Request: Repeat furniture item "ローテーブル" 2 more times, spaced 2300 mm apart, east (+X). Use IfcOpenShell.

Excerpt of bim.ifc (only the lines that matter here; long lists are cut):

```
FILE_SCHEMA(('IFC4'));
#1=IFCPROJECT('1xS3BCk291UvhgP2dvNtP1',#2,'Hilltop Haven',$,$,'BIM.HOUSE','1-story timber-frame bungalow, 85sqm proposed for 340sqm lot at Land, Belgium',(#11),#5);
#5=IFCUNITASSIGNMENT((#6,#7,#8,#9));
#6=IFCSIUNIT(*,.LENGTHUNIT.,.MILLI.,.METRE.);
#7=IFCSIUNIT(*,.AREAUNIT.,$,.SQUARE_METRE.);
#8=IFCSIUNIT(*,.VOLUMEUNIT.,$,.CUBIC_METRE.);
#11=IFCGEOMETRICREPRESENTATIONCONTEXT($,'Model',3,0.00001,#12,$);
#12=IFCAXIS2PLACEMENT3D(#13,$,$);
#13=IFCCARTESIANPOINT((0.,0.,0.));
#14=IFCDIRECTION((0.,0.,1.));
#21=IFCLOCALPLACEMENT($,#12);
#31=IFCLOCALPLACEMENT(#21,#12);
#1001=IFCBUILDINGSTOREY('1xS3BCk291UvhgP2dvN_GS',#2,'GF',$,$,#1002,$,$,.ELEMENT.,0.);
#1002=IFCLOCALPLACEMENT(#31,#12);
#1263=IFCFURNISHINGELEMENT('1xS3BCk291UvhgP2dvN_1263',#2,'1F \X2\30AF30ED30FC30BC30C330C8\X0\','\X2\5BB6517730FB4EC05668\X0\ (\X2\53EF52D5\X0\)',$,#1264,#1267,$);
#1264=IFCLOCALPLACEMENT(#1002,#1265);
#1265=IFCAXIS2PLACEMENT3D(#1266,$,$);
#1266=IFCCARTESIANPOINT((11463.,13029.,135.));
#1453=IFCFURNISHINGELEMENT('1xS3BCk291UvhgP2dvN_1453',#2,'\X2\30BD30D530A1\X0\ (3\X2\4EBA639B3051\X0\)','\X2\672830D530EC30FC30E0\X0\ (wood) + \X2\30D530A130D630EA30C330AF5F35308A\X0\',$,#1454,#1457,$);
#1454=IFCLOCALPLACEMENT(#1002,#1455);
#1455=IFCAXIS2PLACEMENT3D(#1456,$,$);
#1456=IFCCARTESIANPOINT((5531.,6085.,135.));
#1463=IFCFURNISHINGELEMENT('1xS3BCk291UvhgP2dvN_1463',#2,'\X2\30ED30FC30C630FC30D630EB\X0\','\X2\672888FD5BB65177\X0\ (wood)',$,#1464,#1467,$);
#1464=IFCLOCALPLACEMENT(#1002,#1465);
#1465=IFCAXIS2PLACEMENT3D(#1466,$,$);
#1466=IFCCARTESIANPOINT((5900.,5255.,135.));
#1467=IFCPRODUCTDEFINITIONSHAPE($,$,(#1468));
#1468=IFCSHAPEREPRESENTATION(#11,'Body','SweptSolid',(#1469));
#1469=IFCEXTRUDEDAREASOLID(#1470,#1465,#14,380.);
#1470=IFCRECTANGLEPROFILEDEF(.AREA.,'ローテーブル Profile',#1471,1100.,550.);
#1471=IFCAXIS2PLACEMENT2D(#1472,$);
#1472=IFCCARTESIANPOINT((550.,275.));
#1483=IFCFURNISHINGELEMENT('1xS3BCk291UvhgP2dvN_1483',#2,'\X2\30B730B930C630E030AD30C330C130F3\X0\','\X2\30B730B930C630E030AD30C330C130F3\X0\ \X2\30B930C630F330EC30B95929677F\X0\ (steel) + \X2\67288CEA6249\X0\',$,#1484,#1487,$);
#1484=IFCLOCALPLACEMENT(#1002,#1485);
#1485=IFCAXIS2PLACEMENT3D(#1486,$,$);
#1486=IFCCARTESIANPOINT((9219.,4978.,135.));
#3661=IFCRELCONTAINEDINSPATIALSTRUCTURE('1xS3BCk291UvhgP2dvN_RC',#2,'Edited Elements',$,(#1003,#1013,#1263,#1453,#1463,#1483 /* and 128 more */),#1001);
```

```python
import numpy as np
import ifcopenshell
import ifcopenshell.api.geometry
import ifcopenshell.api.root
import ifcopenshell.util.element
import ifcopenshell.util.placement
import ifcopenshell.util.unit

model = ifcopenshell.open("bim.ifc")
unit_scale = ifcopenshell.util.unit.calculate_unit_scale(model)


def reuse_history(source, copy):
    """copy_class also copies each property set's owner history, people and application; keep the originals."""
    for rel in copy.IsDefinedBy:
        if rel.is_a("IfcRelDefinesByProperties") and (history := rel.RelatingPropertyDefinition.OwnerHistory):
            rel.RelatingPropertyDefinition.OwnerHistory = source.OwnerHistory
            ifcopenshell.util.element.remove_deep2(model, history)


source = model.by_guid("1xS3BCk291UvhgP2dvN_1463")
base = ifcopenshell.util.placement.get_local_placement(source.ObjectPlacement)
step = np.array([1.0, 0.0, 0.0]) * 2.3 / unit_scale

for i in range(1, 3):
    copy = ifcopenshell.api.root.copy_class(model, product=source)
    copy.Representation = ifcopenshell.util.element.copy_deep(
        model, source.Representation, exclude=["IfcGeometricRepresentationContext", "IfcRepresentationMap"]
    )
    reuse_history(source, copy)
    matrix = base.copy()
    matrix[:3, 3] += i * step
    print("added at", matrix[:3, 3].round(3) + 0.0)
    ifcopenshell.api.geometry.edit_object_placement(model, product=copy, matrix=matrix, is_si=False)

model.write("bim_v2.ifc")
```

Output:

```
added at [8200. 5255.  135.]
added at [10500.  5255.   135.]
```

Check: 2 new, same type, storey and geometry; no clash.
